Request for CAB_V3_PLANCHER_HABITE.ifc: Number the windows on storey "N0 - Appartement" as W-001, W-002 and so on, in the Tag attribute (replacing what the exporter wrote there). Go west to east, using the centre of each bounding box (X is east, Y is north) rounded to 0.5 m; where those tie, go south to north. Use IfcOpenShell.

First a look at what the model holds.

```python
import ifcopenshell
import ifcopenshell.util.element
import ifcopenshell.util.placement

model = ifcopenshell.open("CAB_V3_PLANCHER_HABITE.ifc")
print(model.schema)
storey = next(s for s in model.by_type("IfcBuildingStorey") if s.Name == "N0 - Appartement")
windows = [e for e in ifcopenshell.util.element.get_decomposition(storey) if e.is_a("IfcWindow")]
for e in sorted(windows, key=lambda e: e.id()):
    origin = ifcopenshell.util.placement.get_local_placement(e.ObjectPlacement)[:3, 3]
    print(e.id(), e.Tag, e.Name, origin.round(2) + 0.0, sep=" | ")
```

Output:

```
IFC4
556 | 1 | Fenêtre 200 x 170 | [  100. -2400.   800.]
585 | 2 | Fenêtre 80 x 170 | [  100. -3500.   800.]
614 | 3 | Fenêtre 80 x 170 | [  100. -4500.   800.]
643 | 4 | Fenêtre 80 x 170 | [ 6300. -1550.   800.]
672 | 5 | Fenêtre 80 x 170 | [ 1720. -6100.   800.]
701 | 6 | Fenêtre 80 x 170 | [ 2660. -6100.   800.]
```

```python
import ifcopenshell
import ifcopenshell.geom
import ifcopenshell.util.element
import ifcopenshell.util.shape

model = ifcopenshell.open("CAB_V3_PLANCHER_HABITE.ifc")
settings = ifcopenshell.geom.settings()
settings.set("use-world-coords", True)


def centre(element):
    shape = ifcopenshell.geom.create_shape(settings, element)
    return ifcopenshell.util.shape.get_bbox_centroid(shape.geometry)


storey = next(s for s in model.by_type("IfcBuildingStorey") if s.Name == "N0 - Appartement")
windows = [e for e in ifcopenshell.util.element.get_decomposition(storey) if e.is_a("IfcWindow")]

# Insertion points can sit at a corner or the storey origin, so sort by the geometry (in metres).
centres = {e: centre(e) for e in windows}
windows.sort(key=lambda e: (round(centres[e][0] / 0.5), centres[e][1]))

for i, e in enumerate(windows, start=1):
    number = f"W-0{i:02d}"
    e.Tag = number
    print(e.id(), number)

model.write("CAB_V3_PLANCHER_HABITE_edited.ifc")
```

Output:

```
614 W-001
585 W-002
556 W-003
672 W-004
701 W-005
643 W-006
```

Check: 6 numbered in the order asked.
